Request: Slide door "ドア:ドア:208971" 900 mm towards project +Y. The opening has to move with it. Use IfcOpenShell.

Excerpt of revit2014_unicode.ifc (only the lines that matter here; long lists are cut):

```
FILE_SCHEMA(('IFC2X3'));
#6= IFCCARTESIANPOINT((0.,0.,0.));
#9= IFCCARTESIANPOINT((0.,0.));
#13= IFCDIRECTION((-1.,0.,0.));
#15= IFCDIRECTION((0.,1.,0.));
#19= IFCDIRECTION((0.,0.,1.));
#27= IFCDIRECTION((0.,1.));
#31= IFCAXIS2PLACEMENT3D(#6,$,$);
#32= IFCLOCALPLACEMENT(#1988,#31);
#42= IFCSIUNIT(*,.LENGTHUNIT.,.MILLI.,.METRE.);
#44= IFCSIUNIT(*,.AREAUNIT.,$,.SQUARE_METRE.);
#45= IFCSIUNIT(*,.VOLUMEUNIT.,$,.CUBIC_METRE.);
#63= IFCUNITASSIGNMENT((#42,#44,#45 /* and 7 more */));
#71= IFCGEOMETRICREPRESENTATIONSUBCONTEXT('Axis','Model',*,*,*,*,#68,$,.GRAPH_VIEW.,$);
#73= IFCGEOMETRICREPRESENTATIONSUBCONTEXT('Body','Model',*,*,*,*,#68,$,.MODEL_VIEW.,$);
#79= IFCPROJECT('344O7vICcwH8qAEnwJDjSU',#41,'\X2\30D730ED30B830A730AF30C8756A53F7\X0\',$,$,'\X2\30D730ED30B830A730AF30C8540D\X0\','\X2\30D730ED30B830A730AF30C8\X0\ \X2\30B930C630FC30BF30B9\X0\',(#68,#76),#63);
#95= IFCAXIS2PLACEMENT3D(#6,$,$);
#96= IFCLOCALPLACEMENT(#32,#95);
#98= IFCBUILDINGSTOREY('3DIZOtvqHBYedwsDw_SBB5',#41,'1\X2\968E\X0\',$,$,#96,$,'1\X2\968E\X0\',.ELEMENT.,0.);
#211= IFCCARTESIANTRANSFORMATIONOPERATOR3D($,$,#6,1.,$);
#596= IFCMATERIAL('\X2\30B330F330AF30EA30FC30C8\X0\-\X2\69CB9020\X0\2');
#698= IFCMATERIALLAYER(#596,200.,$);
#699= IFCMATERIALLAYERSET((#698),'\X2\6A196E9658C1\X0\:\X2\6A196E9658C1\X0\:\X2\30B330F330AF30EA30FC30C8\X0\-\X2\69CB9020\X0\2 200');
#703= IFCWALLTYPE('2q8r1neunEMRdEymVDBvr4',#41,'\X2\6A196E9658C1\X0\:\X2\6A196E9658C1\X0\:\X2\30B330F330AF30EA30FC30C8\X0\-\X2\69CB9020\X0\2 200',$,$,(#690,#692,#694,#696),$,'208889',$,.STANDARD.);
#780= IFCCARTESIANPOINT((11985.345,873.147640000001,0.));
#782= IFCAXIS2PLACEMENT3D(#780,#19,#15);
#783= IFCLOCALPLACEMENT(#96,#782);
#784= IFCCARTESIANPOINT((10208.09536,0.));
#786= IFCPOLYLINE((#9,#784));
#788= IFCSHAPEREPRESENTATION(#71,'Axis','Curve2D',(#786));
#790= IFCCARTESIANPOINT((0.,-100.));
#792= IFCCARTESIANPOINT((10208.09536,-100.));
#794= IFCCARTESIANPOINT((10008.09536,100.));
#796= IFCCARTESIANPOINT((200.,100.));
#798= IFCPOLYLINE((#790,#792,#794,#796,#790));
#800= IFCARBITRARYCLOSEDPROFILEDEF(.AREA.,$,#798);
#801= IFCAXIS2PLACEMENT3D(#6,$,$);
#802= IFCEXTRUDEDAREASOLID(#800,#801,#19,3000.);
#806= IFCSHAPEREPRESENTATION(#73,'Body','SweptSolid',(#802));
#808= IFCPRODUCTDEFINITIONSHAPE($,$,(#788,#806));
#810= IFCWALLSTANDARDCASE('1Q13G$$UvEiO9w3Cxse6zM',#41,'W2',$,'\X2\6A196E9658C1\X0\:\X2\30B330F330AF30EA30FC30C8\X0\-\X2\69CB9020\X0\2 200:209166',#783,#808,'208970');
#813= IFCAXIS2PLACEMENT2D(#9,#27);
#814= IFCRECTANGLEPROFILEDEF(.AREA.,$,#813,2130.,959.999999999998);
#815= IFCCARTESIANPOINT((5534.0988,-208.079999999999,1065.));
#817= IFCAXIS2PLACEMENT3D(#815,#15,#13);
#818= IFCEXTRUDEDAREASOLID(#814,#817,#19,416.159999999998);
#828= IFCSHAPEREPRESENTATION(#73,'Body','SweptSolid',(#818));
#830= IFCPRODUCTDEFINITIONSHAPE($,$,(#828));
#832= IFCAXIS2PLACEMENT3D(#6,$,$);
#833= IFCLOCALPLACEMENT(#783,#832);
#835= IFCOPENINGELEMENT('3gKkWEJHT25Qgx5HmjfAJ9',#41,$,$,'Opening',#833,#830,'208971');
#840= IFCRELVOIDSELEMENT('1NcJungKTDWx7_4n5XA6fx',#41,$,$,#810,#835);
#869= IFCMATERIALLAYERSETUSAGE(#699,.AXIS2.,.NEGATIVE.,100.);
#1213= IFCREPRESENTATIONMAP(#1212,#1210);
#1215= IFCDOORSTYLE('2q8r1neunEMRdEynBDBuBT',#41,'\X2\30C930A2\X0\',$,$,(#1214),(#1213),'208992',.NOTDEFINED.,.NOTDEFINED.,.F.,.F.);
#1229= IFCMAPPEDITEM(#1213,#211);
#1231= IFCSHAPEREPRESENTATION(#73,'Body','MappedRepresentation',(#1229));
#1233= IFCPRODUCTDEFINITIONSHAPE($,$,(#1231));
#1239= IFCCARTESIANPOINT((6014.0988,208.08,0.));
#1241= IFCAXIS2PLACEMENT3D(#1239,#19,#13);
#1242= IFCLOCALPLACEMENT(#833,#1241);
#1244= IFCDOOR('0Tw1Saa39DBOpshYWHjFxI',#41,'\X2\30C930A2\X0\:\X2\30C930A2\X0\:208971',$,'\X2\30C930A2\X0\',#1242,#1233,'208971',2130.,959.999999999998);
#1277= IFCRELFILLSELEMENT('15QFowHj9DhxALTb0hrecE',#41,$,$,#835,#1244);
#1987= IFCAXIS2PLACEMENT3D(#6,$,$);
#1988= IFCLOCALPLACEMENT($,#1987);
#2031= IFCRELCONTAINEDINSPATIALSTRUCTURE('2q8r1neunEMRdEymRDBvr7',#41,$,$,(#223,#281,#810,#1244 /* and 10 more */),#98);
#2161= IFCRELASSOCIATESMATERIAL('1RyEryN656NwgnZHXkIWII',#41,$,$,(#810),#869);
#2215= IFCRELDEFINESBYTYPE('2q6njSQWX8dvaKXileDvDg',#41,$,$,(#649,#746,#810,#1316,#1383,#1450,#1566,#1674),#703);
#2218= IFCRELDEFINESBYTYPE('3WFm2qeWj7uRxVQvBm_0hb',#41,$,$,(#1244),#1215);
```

```python
import ifcopenshell
import ifcopenshell.api.geometry
import ifcopenshell.util.placement
import ifcopenshell.util.unit

model = ifcopenshell.open("revit2014_unicode.ifc")
unit_scale = ifcopenshell.util.unit.calculate_unit_scale(model)

door = model.by_guid("0Tw1Saa39DBOpshYWHjFxI")
opening = door.FillsVoids[0].RelatingOpeningElement
wall = opening.VoidsElements[0].RelatingBuildingElement

wall_matrix = ifcopenshell.util.placement.get_local_placement(wall.ObjectPlacement)
shift = wall_matrix[:3, 0] * 0.9 / unit_scale
before = ifcopenshell.util.placement.get_local_placement(door.ObjectPlacement)[:3, 3].copy()

# The door is placed relative to its opening, so it follows when the opening moves.
matrix = ifcopenshell.util.placement.get_local_placement(opening.ObjectPlacement)
matrix[:3, 3] += shift
ifcopenshell.api.geometry.edit_object_placement(
    model, product=opening, matrix=matrix, is_si=False, should_transform_children=True
)

after = ifcopenshell.util.placement.get_local_placement(door.ObjectPlacement)[:3, 3]
print("door moved by", (after - before).round(3) + 0.0)

model.write("revit2014_unicode_v2.ifc")
```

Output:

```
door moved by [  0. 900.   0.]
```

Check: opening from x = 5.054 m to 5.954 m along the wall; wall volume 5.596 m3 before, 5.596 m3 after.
